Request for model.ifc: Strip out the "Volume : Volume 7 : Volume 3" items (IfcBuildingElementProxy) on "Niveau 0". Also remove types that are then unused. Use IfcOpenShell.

First a look at what the model holds.

```python
import ifcopenshell
import ifcopenshell.util.element

model = ifcopenshell.open("model.ifc")
print(model.schema)
storey = next(s for s in model.by_type("IfcBuildingStorey") if s.Name == "Niveau 0")
proxies = [e for e in ifcopenshell.util.element.get_decomposition(storey) if e.is_a("IfcBuildingElementProxy")]
seen = {}
for e in proxies:
    element_type = ifcopenshell.util.element.get_type(e)
    name = element_type.Name if element_type not in (None, e) else None
    seen[name] = seen.get(name, 0) + 1
for name, count in sorted(seen.items(), key=str):
    print(count, "x", name)
```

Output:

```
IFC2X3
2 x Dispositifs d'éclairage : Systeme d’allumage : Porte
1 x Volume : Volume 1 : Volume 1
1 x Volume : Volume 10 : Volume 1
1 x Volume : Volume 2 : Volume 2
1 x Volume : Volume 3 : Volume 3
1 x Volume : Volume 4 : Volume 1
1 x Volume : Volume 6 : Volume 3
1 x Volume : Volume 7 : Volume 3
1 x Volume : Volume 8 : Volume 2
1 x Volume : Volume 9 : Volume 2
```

```python
import ifcopenshell
import ifcopenshell.api.root
import ifcopenshell.util.element

model = ifcopenshell.open("model.ifc")

storey = next(s for s in model.by_type("IfcBuildingStorey") if s.Name == "Niveau 0")
proxies = [e for e in ifcopenshell.util.element.get_decomposition(storey) if e.is_a("IfcBuildingElementProxy")]
targets = [e for e in proxies if (t := ifcopenshell.util.element.get_type(e)) not in (None, e) and t.Name == "Volume : Volume 7 : Volume 3"]
types = {ifcopenshell.util.element.get_type(e) for e in targets} - {None, *targets}

for e in targets:
    ifcopenshell.api.root.remove_product(model, product=e)
print(len(targets), "removed")

unused = [t for t in types if not ifcopenshell.util.element.get_types(t)]
for t in unused:
    ifcopenshell.api.root.remove_product(model, product=t)
print(len(unused), "unused types removed")

model.write("model-out.ifc")
```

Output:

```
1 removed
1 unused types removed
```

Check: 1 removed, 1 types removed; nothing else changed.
